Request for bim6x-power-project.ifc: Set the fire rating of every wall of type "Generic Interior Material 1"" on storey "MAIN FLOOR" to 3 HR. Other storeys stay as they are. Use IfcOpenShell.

First a look at what the model holds.

```python
import ifcopenshell
import ifcopenshell.util.element

model = ifcopenshell.open("bim6x-power-project.ifc")
print(model.schema)
storey = next(s for s in model.by_type("IfcBuildingStorey") if s.Name == "MAIN FLOOR")
walls = [e for e in ifcopenshell.util.element.get_decomposition(storey) if e.is_a("IfcWall")]
seen = {}
for e in walls:
    element_type = ifcopenshell.util.element.get_type(e)
    key = (element_type.Name if element_type != e and element_type else None, ifcopenshell.util.element.get_pset(e, "Pset_WallCommon", "FireRating"))
    seen[key] = seen.get(key, 0) + 1
for (name, value), count in sorted(seen.items(), key=str):
    print(count, "x", name, "|", value)
```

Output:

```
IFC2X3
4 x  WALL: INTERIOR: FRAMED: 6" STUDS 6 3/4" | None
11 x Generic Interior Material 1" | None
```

```python
import ifcopenshell
import ifcopenshell.api.pset
import ifcopenshell.util.element

model = ifcopenshell.open("bim6x-power-project.ifc")

storey = next(s for s in model.by_type("IfcBuildingStorey") if s.Name == "MAIN FLOOR")
walls = [e for e in ifcopenshell.util.element.get_decomposition(storey) if e.is_a("IfcWall")]

count = 0
for e in walls:
    element_type = ifcopenshell.util.element.get_type(e)
    if element_type in (None, e) or element_type.Name != 'Generic Interior Material 1"':
        continue
    # add_pset returns the element's existing set when there is one.
    pset = ifcopenshell.api.pset.add_pset(model, product=e, name="Pset_WallCommon")
    ifcopenshell.api.pset.edit_pset(model, pset=pset, properties={"FireRating": "3 HR"})
    count += 1

print(count, "walls updated")

model.write("bim6x-power-project_rev.ifc")
```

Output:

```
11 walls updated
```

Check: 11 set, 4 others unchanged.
